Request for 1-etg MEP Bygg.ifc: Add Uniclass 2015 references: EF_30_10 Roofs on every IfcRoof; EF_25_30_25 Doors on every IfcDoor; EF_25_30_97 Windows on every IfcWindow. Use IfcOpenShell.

First a look at what the model holds.

```python
import ifcopenshell

model = ifcopenshell.open("1-etg MEP Bygg.ifc")
print(model.schema)
print("classifications:", [c.Name for c in model.by_type("IfcClassification")])
for ifc_class in ("IfcDoor", "IfcRoof", "IfcStair", "IfcWall", "IfcWindow"):
    print(ifc_class, len(model.by_type(ifc_class)))
```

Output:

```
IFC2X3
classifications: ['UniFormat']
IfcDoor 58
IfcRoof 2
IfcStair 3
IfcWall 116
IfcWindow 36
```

```python
import ifcopenshell
import ifcopenshell.api.classification

model = ifcopenshell.open("1-etg MEP Bygg.ifc")

# IFC2X3 requires Source and Edition and has no link from the project to the system.
system = model.create_entity("IfcClassification", Source="NBS", Edition="2015", Name="Uniclass 2015")

codes = {
    "IfcRoof": ("EF_30_10", "Roofs"),
    "IfcDoor": ("EF_25_30_25", "Doors"),
    "IfcWindow": ("EF_25_30_97", "Windows"),
}
for ifc_class, (code, name) in codes.items():
    products = model.by_type(ifc_class)
    ifcopenshell.api.classification.add_reference(
        model, products=products, classification=system, identification=code, name=name
    )
    print(code, len(products))

model.write("1-etg MEP Bygg-out.ifc")
```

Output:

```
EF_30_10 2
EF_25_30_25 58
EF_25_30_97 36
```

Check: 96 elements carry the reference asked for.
